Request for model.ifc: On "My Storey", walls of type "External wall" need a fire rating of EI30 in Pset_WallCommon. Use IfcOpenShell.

First a look at what the model holds.

```python
import ifcopenshell
import ifcopenshell.util.element

model = ifcopenshell.open("model.ifc")
print(model.schema)
storey = next(s for s in model.by_type("IfcBuildingStorey") if s.Name == "My Storey")
walls = [e for e in ifcopenshell.util.element.get_decomposition(storey) if e.is_a("IfcWall")]
seen = {}
for e in walls:
    element_type = ifcopenshell.util.element.get_type(e)
    key = (element_type.Name if element_type != e and element_type else None, ifcopenshell.util.element.get_pset(e, "Pset_WallCommon", "FireRating"))
    seen[key] = seen.get(key, 0) + 1
for (name, value), count in sorted(seen.items(), key=str):
    print(count, "x", name, "|", value)
```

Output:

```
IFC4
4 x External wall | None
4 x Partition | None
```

```python
import ifcopenshell
import ifcopenshell.api.pset
import ifcopenshell.util.element

model = ifcopenshell.open("model.ifc")

storey = next(s for s in model.by_type("IfcBuildingStorey") if s.Name == "My Storey")
walls = [e for e in ifcopenshell.util.element.get_decomposition(storey) if e.is_a("IfcWall")]

count = 0
for e in walls:
    element_type = ifcopenshell.util.element.get_type(e)
    if element_type in (None, e) or element_type.Name != "External wall":
        continue
    # add_pset returns the element's existing set when there is one.
    pset = ifcopenshell.api.pset.add_pset(model, product=e, name="Pset_WallCommon")
    ifcopenshell.api.pset.edit_pset(model, pset=pset, properties={"FireRating": "EI30"})
    count += 1

print(count, "walls updated")

model.write("model_edited.ifc")
```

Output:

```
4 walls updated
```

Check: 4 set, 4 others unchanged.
